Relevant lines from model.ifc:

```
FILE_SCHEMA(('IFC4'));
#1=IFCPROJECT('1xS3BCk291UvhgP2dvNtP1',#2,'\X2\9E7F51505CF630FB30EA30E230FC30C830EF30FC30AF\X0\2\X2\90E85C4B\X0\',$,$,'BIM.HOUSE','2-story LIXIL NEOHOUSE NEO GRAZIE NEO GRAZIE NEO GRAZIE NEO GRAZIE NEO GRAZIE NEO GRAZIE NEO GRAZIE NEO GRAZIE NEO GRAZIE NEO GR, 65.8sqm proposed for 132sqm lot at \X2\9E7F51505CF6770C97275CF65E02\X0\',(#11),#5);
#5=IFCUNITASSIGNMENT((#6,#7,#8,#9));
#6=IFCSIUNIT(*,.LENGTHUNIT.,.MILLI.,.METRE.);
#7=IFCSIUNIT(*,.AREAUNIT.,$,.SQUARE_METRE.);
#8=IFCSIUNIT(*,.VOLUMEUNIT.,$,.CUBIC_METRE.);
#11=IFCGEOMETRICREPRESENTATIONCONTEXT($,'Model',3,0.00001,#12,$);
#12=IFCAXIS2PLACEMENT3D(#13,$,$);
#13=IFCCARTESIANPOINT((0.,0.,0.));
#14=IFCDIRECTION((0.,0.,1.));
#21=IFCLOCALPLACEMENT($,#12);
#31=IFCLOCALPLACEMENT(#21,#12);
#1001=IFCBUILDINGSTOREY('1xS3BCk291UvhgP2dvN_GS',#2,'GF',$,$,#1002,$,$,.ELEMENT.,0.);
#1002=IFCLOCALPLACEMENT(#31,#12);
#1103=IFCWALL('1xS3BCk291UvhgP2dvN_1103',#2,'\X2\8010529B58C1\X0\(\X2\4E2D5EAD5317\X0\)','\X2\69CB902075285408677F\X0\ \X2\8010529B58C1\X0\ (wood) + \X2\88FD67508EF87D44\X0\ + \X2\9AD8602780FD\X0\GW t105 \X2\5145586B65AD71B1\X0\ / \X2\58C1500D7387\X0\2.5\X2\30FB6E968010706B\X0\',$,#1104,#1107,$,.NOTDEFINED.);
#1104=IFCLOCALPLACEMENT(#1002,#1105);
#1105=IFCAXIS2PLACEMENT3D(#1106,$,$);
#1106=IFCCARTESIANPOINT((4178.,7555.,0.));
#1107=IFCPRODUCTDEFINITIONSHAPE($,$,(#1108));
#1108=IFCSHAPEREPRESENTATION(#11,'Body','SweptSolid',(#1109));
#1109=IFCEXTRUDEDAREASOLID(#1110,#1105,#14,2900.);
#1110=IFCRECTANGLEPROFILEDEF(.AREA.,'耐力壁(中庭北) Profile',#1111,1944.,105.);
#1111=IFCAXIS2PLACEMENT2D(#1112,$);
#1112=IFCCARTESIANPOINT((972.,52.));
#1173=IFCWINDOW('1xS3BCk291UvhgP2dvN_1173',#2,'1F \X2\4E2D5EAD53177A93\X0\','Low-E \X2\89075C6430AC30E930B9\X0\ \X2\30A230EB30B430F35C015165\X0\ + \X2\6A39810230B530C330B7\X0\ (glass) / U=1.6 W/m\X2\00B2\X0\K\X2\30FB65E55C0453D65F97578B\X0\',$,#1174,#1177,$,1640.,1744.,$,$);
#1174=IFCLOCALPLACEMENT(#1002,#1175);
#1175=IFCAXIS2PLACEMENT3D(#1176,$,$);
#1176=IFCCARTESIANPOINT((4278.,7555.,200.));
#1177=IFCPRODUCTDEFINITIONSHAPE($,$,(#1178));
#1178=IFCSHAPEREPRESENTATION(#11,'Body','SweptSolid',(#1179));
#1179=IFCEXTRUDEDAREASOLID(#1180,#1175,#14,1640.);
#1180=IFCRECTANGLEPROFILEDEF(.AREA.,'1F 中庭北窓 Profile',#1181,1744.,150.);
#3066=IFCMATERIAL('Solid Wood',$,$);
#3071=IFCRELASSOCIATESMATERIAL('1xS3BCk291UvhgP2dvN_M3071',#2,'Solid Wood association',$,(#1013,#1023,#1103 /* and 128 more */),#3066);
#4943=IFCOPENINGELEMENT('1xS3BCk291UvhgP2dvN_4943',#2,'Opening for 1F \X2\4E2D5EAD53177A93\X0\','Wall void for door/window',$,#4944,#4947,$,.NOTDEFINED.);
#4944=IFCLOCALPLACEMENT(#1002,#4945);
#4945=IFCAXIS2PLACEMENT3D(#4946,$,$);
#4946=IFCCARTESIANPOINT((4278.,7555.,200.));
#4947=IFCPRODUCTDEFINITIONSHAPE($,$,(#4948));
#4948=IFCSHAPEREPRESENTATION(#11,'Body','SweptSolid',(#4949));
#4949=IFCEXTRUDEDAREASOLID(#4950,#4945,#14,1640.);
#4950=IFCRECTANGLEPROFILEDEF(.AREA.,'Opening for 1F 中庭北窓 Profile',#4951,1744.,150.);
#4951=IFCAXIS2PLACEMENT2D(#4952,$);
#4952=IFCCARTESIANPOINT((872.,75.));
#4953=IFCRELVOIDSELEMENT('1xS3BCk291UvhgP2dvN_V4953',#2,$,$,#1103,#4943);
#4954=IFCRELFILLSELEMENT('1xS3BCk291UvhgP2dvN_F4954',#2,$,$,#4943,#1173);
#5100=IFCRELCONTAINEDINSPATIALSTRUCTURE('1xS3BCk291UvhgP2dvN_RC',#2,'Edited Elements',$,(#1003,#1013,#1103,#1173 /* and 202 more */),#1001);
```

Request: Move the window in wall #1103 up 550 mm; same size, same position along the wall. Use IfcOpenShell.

```python
import numpy as np
import ifcopenshell
import ifcopenshell.api.geometry
import ifcopenshell.util.placement
import ifcopenshell.util.unit

model = ifcopenshell.open("model.ifc")
unit_scale = ifcopenshell.util.unit.calculate_unit_scale(model)

window = model.by_guid("1xS3BCk291UvhgP2dvN_1173")
opening = window.FillsVoids[0].RelatingOpeningElement
dz = 550.0

shift = np.array([0.0, 0.0, dz])
# The window is not placed relative to its opening, so move both.
for product in (opening, window):
    matrix = ifcopenshell.util.placement.get_local_placement(product.ObjectPlacement)
    matrix[:3, 3] += shift
    ifcopenshell.api.geometry.edit_object_placement(model, product=product, matrix=matrix, is_si=False)

print(f"moved by {dz * unit_scale:+.3f} m")

model.write("model_edited.ifc")
```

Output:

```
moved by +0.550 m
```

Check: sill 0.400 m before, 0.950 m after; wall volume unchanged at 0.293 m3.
